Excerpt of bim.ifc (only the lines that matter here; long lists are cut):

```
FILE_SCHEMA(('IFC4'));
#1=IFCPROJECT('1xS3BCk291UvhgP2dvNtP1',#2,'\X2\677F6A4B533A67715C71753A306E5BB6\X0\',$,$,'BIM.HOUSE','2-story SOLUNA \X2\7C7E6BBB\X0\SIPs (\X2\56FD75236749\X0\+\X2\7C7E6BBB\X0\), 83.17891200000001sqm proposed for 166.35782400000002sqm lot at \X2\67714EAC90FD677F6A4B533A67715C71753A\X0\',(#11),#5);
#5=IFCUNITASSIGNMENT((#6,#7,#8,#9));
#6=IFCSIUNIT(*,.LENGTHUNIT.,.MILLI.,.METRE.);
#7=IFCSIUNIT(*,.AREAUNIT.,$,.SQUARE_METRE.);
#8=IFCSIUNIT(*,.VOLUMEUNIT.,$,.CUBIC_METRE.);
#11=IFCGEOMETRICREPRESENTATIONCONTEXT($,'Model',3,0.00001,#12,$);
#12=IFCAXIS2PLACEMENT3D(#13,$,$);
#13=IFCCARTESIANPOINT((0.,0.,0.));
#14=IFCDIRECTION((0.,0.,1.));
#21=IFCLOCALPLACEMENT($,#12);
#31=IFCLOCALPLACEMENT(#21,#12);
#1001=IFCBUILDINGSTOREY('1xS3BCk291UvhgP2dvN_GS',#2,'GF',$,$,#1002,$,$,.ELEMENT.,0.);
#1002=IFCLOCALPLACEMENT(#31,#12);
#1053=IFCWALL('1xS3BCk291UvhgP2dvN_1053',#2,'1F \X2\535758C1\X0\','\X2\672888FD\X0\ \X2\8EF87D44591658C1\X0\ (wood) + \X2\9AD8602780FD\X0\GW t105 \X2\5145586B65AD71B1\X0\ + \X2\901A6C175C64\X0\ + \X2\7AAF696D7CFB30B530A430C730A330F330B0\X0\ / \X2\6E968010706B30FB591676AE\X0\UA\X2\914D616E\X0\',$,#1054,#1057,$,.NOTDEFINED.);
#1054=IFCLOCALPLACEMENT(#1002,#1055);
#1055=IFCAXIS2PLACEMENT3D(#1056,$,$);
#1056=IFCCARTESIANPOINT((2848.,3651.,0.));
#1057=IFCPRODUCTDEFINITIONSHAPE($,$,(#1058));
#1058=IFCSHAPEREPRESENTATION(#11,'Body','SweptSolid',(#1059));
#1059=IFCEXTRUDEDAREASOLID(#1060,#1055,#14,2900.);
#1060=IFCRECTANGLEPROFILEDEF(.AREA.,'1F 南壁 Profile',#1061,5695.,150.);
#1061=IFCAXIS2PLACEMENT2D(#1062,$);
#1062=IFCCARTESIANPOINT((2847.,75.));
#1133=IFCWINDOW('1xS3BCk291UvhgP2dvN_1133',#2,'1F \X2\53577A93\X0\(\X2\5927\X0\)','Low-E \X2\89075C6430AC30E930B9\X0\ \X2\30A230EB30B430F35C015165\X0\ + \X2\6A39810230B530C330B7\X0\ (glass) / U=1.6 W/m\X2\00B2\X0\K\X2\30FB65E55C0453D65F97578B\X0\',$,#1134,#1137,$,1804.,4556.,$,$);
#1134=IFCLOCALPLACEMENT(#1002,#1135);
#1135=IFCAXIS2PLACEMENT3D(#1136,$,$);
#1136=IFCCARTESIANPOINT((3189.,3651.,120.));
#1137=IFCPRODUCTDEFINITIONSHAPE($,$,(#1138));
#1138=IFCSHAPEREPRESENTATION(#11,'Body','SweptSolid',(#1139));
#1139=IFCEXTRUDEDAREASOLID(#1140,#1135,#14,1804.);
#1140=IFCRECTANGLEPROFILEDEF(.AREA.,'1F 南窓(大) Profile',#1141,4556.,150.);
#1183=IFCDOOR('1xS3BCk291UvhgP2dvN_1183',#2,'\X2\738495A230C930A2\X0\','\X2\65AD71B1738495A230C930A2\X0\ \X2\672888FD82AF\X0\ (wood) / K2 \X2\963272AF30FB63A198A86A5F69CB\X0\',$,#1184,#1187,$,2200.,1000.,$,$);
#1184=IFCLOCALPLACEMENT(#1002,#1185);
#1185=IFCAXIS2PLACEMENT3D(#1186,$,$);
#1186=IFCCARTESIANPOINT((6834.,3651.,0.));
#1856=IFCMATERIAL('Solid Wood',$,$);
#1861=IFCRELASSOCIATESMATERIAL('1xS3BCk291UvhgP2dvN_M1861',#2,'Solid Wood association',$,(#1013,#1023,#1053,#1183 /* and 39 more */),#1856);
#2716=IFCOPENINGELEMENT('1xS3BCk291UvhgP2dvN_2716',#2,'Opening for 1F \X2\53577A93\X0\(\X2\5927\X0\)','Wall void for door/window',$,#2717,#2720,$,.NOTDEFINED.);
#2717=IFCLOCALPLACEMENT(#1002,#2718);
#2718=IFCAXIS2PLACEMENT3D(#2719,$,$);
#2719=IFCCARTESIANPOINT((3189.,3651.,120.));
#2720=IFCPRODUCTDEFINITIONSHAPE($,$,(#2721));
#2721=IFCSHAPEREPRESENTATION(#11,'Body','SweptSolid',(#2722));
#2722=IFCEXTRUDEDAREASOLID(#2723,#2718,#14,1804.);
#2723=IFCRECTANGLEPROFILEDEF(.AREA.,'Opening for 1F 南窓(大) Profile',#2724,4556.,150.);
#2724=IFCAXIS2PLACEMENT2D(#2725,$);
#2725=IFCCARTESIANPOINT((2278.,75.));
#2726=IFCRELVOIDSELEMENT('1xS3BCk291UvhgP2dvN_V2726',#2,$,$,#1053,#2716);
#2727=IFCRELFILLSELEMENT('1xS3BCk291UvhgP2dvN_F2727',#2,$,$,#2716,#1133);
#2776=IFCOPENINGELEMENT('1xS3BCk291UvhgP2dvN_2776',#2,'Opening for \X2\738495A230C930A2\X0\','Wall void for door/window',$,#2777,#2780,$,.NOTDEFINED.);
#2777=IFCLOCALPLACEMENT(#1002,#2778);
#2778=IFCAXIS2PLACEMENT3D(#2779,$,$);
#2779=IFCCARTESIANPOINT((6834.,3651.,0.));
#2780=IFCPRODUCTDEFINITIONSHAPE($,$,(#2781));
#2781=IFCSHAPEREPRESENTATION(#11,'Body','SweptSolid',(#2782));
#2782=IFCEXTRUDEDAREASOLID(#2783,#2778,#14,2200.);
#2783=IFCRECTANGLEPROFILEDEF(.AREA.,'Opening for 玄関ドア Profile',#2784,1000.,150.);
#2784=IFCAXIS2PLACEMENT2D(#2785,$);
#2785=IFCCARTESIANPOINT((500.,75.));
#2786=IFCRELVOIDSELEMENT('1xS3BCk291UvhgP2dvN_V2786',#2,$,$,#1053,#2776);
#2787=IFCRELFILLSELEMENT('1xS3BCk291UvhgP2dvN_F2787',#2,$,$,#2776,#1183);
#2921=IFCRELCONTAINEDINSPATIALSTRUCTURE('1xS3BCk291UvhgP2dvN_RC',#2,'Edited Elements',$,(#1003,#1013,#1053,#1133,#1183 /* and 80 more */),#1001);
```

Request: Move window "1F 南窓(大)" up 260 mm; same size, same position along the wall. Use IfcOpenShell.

```python
import numpy as np
import ifcopenshell
import ifcopenshell.api.geometry
import ifcopenshell.util.placement
import ifcopenshell.util.unit

model = ifcopenshell.open("bim.ifc")
unit_scale = ifcopenshell.util.unit.calculate_unit_scale(model)

window = model.by_id(1133)
opening = window.FillsVoids[0].RelatingOpeningElement
dz = 0.26 / unit_scale

shift = np.array([0.0, 0.0, dz])
# The window is not placed relative to its opening, so move both.
for product in (opening, window):
    matrix = ifcopenshell.util.placement.get_local_placement(product.ObjectPlacement)
    matrix[:3, 3] += shift
    ifcopenshell.api.geometry.edit_object_placement(model, product=product, matrix=matrix, is_si=False)

print(f"moved by {dz * unit_scale:+.3f} m")

model.write("bim_edited.ifc")
```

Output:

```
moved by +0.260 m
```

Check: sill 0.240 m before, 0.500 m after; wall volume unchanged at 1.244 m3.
